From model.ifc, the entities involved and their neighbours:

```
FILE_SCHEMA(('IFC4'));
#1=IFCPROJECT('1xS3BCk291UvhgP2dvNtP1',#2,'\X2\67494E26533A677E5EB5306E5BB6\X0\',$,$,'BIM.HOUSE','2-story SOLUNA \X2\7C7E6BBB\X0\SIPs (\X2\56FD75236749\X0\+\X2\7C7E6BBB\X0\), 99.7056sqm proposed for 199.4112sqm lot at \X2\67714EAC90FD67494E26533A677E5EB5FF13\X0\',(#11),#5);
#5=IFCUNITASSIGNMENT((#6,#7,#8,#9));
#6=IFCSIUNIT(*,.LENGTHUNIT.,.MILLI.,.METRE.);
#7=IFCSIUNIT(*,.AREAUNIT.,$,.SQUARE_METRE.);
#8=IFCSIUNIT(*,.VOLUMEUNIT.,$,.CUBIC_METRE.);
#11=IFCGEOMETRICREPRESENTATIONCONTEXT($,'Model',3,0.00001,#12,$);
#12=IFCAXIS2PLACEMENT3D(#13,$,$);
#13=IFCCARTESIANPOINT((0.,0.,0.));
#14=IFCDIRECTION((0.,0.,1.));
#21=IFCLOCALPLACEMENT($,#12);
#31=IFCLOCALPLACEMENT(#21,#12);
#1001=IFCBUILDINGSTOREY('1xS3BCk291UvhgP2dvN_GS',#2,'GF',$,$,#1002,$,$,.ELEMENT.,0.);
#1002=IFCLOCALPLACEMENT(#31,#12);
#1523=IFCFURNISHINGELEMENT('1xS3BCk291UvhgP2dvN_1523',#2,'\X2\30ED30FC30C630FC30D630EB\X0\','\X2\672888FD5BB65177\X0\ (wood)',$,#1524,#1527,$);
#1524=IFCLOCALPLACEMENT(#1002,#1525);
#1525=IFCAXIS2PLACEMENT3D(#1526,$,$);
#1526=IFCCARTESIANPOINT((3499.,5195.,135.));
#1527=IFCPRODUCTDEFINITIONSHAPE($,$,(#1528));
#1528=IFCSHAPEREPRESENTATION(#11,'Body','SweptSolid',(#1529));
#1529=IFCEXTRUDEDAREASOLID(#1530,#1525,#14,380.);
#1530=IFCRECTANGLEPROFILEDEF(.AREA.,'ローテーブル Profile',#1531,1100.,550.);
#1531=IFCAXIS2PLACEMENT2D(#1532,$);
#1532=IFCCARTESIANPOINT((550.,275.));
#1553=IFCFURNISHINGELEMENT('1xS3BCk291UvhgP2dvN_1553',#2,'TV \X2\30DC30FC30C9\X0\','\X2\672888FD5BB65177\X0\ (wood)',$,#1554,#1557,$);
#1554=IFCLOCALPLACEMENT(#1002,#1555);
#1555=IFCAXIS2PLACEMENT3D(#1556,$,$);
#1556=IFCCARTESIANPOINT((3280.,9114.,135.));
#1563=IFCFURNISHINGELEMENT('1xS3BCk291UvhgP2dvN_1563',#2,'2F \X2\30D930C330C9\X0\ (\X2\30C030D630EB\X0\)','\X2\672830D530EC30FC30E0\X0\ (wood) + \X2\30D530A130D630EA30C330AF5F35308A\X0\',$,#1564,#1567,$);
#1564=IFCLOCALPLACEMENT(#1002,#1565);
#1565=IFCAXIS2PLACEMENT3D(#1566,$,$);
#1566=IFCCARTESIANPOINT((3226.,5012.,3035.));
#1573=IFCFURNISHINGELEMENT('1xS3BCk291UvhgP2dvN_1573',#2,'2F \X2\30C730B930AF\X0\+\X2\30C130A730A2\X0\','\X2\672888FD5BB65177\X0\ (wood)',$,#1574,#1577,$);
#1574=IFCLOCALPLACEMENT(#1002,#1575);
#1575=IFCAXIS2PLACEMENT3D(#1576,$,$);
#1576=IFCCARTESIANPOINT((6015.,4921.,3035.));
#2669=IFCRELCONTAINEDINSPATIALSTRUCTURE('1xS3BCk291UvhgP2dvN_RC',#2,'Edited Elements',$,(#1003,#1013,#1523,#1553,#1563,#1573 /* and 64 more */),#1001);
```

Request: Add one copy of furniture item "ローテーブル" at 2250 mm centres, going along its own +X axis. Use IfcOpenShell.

```python
import ifcopenshell
import ifcopenshell.api.geometry
import ifcopenshell.api.root
import ifcopenshell.util.element
import ifcopenshell.util.placement

model = ifcopenshell.open("model.ifc")


def reuse_history(source, copy):
    """copy_class also copies each property set's owner history, people and application; keep the originals."""
    for rel in copy.IsDefinedBy:
        if rel.is_a("IfcRelDefinesByProperties") and (history := rel.RelatingPropertyDefinition.OwnerHistory):
            rel.RelatingPropertyDefinition.OwnerHistory = source.OwnerHistory
            ifcopenshell.util.element.remove_deep2(model, history)


source = model.by_guid("1xS3BCk291UvhgP2dvN_1523")
base = ifcopenshell.util.placement.get_local_placement(source.ObjectPlacement)
step = base[:3, 0] * 2250.0

for i in range(1, 2):
    copy = ifcopenshell.api.root.copy_class(model, product=source)
    copy.Representation = ifcopenshell.util.element.copy_deep(
        model, source.Representation, exclude=["IfcGeometricRepresentationContext", "IfcRepresentationMap"]
    )
    reuse_history(source, copy)
    matrix = base.copy()
    matrix[:3, 3] += i * step
    print("added at", matrix[:3, 3].round(3) + 0.0)
    ifcopenshell.api.geometry.edit_object_placement(model, product=copy, matrix=matrix, is_si=False)

model.write("model-out.ifc")
```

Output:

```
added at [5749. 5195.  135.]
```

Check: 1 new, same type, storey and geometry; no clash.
